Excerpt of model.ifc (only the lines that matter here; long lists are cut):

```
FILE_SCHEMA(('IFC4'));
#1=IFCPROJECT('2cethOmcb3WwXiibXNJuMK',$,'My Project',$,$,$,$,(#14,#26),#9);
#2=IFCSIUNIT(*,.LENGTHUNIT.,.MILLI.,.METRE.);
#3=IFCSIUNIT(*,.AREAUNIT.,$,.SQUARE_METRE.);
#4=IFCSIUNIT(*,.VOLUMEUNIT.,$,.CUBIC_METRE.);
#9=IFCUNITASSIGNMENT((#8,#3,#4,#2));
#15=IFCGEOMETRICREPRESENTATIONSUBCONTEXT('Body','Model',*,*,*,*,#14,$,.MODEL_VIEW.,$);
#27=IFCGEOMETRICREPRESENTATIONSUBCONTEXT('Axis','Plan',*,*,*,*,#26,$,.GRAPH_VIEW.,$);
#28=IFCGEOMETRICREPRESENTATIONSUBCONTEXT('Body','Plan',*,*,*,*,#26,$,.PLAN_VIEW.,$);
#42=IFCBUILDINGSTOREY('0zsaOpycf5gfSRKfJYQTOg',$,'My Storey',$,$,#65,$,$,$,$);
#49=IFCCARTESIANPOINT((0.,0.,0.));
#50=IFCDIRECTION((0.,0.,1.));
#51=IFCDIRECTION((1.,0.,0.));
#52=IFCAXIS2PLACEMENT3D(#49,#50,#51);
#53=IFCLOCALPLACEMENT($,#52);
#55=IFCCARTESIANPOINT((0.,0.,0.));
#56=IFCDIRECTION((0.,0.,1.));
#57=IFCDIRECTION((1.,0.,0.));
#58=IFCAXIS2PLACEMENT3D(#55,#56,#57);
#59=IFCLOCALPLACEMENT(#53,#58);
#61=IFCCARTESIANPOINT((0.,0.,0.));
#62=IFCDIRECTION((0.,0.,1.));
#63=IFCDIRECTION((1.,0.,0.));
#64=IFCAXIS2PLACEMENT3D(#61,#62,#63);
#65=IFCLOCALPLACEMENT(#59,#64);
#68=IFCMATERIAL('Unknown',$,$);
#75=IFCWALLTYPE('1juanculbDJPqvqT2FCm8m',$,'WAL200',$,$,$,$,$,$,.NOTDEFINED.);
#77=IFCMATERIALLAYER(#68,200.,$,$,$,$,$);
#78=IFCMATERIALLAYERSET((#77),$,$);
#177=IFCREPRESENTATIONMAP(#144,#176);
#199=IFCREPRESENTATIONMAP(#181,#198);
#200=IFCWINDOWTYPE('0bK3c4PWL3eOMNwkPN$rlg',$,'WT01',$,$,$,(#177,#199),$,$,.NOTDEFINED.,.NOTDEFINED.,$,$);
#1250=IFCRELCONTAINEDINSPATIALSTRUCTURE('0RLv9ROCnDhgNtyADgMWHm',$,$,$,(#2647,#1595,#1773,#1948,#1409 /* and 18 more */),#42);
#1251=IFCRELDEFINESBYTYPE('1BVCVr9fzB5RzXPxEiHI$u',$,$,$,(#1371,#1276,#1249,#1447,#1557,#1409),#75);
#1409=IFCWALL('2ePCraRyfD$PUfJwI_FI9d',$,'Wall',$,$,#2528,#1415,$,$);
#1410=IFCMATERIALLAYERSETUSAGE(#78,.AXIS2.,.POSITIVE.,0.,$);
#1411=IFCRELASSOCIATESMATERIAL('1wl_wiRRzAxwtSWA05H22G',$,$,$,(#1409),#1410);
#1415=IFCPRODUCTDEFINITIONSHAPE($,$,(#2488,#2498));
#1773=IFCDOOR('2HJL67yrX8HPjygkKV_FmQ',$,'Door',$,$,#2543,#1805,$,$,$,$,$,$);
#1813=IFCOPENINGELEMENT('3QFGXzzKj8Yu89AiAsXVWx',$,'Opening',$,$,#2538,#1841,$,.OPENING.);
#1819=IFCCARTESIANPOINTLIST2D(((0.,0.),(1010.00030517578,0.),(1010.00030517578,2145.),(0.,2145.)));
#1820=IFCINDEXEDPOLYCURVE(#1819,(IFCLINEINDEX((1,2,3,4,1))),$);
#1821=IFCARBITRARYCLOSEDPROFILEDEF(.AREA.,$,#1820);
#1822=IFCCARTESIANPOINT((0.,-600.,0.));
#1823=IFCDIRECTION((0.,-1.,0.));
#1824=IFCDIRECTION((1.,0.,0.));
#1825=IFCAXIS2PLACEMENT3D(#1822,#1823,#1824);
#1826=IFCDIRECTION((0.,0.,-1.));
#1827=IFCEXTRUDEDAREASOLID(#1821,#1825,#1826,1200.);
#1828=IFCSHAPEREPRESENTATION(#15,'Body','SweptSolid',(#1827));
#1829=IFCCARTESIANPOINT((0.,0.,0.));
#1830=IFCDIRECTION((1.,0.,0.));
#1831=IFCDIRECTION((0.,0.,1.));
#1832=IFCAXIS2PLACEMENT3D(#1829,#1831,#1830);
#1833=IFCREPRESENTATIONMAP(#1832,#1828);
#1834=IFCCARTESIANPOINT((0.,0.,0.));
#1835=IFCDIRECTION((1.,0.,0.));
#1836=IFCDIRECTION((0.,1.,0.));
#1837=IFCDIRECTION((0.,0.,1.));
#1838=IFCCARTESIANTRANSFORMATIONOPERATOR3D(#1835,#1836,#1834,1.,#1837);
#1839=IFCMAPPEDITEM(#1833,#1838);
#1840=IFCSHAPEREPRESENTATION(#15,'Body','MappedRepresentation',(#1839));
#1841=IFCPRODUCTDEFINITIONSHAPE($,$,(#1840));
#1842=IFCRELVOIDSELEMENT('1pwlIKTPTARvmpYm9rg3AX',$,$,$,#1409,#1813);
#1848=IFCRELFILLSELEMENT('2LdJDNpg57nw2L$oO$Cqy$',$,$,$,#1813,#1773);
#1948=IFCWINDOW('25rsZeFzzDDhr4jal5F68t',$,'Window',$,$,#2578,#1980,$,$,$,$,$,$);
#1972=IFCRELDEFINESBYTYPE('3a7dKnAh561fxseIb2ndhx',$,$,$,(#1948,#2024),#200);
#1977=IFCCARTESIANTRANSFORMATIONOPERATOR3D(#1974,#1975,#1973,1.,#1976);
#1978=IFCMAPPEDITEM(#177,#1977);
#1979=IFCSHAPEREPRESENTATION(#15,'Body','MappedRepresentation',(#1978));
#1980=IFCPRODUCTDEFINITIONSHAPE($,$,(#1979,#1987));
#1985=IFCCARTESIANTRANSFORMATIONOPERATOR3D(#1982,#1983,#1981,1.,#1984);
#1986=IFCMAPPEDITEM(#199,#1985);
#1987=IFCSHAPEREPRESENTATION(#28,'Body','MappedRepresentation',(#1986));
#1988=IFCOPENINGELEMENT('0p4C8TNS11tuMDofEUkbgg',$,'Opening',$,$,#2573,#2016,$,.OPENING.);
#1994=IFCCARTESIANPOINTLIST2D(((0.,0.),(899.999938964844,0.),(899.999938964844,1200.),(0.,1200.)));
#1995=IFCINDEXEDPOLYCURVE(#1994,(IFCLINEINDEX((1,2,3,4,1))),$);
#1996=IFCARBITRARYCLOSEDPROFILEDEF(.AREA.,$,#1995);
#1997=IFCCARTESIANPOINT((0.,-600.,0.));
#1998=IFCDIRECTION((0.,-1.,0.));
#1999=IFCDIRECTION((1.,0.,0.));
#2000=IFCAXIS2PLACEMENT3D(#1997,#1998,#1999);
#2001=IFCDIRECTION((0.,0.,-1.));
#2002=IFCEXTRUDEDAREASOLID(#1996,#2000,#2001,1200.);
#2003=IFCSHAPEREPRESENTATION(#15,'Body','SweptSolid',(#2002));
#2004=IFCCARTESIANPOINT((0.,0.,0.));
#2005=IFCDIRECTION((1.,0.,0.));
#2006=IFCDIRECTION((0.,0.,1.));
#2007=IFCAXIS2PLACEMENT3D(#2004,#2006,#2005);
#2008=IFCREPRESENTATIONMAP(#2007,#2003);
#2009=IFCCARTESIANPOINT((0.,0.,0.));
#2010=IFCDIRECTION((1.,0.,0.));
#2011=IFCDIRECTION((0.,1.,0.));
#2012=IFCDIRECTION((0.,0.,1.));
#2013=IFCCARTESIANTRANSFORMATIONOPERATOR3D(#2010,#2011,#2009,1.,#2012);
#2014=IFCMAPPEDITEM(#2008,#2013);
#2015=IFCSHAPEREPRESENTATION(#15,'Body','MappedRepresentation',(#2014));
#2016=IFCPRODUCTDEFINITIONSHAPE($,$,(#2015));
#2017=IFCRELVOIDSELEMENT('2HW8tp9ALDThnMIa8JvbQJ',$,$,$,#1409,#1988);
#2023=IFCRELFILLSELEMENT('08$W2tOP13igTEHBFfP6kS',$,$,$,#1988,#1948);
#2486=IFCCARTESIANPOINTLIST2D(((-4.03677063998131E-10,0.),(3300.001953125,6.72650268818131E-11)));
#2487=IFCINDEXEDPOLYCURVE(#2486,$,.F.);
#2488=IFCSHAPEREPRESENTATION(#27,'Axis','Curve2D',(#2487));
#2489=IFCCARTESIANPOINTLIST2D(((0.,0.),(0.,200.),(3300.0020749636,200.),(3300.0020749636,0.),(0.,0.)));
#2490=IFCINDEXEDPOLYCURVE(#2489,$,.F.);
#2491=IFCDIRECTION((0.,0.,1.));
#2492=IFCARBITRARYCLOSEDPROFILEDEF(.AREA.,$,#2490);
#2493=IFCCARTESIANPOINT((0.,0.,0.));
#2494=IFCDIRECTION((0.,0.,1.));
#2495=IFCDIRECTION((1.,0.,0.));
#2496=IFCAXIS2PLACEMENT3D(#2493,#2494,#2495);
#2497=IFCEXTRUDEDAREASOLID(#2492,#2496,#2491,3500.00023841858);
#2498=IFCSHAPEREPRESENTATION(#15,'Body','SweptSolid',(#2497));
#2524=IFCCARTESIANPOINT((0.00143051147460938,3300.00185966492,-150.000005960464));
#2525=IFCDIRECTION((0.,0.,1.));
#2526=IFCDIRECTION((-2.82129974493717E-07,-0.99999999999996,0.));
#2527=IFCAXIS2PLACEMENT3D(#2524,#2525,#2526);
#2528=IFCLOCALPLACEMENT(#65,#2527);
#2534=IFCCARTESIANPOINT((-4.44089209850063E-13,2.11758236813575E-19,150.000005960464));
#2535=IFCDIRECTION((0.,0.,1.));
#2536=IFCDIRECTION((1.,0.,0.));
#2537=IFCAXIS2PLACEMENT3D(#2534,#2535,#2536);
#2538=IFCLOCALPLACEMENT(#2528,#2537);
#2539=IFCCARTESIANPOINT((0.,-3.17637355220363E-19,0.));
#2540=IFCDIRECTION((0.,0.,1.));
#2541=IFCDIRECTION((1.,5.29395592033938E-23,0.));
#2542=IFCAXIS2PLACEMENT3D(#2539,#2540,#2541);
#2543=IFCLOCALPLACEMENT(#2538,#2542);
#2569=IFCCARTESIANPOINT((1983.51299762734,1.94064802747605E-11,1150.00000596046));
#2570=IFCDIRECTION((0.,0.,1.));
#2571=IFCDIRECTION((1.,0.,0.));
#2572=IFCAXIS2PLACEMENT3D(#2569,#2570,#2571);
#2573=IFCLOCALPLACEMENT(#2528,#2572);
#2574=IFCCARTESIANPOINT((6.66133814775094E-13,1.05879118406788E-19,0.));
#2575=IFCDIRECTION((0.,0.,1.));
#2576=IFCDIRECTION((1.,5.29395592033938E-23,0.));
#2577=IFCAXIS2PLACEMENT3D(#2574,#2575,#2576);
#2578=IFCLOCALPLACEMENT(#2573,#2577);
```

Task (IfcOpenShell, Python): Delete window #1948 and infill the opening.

```python
import ifcopenshell
import ifcopenshell.api.feature
import ifcopenshell.api.root
import ifcopenshell.geom
import ifcopenshell.util.shape

model = ifcopenshell.open("model.ifc")
settings = ifcopenshell.geom.settings()


def volume(element):
    """Net volume in cubic metres, openings subtracted."""
    shape = ifcopenshell.geom.create_shape(settings, element)
    return ifcopenshell.util.shape.get_volume(shape.geometry)


window = model.by_guid("25rsZeFzzDDhr4jal5F68t")
opening = window.FillsVoids[0].RelatingOpeningElement
wall = opening.VoidsElements[0].RelatingBuildingElement
before = volume(wall)

ifcopenshell.api.root.remove_product(model, product=window)
ifcopenshell.api.feature.remove_feature(model, feature=opening)

after = volume(wall)

print(f"wall volume {before:.3f} -> {after:.3f} m3")

model.write("model_v2.ifc")
```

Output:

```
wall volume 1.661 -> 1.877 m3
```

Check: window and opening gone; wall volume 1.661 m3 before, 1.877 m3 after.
